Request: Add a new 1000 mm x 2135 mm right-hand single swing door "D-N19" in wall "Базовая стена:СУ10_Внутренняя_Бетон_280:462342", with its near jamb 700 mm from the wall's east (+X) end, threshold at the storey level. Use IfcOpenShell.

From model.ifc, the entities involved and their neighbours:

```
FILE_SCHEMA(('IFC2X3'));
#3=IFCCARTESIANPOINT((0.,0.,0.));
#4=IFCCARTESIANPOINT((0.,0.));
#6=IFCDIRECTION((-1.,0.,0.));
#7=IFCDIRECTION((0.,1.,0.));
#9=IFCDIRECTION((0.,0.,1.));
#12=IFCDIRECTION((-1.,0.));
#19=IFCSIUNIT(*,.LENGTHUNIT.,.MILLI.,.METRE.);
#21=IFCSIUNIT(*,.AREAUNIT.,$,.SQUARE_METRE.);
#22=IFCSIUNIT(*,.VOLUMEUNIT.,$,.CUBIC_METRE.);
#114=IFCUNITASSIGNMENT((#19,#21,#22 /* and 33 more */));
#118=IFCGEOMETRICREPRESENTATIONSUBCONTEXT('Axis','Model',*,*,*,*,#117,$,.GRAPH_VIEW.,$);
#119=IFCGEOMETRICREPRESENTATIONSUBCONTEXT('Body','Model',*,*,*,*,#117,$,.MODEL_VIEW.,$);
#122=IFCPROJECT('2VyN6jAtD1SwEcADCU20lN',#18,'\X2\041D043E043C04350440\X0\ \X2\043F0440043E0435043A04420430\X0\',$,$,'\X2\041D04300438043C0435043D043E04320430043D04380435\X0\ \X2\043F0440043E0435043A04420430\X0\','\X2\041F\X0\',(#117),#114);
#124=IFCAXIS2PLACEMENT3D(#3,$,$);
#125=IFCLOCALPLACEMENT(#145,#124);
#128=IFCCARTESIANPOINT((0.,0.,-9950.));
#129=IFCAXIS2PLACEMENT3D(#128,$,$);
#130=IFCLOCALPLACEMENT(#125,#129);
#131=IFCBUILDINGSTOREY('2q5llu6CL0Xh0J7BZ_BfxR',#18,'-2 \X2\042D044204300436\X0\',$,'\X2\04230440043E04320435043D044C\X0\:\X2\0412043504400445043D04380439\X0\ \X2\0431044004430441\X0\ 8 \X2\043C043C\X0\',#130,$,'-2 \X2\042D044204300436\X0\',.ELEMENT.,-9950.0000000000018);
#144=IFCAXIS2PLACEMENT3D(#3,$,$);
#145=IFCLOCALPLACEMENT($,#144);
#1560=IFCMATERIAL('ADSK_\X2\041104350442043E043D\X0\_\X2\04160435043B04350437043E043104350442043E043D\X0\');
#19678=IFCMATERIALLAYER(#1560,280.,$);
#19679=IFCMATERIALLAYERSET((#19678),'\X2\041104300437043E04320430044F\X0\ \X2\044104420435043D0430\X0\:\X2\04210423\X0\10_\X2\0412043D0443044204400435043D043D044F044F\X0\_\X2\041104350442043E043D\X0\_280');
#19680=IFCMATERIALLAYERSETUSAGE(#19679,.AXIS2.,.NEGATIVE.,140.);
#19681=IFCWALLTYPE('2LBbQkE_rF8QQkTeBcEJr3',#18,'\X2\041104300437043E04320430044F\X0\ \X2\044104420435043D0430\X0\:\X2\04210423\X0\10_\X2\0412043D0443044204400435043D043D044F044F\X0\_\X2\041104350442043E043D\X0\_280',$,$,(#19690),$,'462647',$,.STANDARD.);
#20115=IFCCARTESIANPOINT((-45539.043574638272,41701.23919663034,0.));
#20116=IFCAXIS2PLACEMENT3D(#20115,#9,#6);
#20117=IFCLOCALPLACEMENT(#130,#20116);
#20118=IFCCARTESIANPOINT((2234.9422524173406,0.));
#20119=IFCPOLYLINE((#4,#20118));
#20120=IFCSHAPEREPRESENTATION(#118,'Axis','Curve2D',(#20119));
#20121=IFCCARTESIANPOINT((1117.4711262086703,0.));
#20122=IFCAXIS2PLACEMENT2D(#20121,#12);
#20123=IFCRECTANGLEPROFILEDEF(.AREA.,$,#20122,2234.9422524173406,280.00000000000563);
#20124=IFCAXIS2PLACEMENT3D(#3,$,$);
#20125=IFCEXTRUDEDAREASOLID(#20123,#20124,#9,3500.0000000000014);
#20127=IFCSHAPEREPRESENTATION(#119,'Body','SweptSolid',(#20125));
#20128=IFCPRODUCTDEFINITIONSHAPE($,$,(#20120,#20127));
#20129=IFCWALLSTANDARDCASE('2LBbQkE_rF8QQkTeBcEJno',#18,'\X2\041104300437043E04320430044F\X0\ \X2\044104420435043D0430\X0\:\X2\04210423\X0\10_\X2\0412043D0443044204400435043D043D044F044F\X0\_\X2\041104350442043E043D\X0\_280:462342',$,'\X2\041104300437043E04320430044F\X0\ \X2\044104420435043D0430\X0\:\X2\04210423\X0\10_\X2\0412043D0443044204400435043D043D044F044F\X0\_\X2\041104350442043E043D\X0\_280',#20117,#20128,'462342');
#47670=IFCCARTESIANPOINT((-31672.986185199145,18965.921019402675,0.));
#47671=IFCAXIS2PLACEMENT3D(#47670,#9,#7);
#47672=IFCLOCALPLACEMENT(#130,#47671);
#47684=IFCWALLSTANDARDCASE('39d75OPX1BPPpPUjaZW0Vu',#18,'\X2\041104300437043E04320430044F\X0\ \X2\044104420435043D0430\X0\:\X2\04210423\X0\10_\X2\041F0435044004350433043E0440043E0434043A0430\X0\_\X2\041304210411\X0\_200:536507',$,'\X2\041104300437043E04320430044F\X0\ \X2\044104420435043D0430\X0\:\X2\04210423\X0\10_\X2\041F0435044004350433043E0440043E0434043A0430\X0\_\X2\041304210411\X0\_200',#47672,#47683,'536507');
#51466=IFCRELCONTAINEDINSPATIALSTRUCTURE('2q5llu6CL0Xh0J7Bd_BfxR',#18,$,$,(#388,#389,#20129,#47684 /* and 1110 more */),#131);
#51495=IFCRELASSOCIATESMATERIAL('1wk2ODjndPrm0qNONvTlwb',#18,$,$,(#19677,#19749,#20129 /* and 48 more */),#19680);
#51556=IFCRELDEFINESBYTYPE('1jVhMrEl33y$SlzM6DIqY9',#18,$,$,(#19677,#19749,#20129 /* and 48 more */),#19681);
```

```python
import numpy as np
import ifcopenshell
import ifcopenshell.api.feature
import ifcopenshell.api.geometry
import ifcopenshell.api.root
import ifcopenshell.api.spatial
import ifcopenshell.api.type
import ifcopenshell.geom
import ifcopenshell.util.element
import ifcopenshell.util.placement
import ifcopenshell.util.representation
import ifcopenshell.util.shape
import ifcopenshell.util.unit

model = ifcopenshell.open("model.ifc")
unit_scale = ifcopenshell.util.unit.calculate_unit_scale(model)
settings = ifcopenshell.geom.settings()


def volume(element):
    """Net volume in cubic metres, openings subtracted."""
    shape = ifcopenshell.geom.create_shape(settings, element)
    return ifcopenshell.util.shape.get_volume(shape.geometry)


wall = model.by_guid("2LBbQkE_rF8QQkTeBcEJno")
storey = ifcopenshell.util.element.get_container(wall, ifc_class="IfcBuildingStorey")
context = ifcopenshell.util.representation.get_context(model, "Model", "Body", "MODEL_VIEW")
before = volume(wall)

width, height, from_end, sill = 1, 2.135, 0.7, 0.0  # metres

# The wall runs along its own X axis, and the end named is its -X end.
wall_shape = ifcopenshell.geom.create_shape(settings, wall)
x, y, z = ifcopenshell.util.shape.get_vertices(wall_shape.geometry).T
start = x.min() + from_end
face, thickness = float(y.min()), float(y.max() - y.min())
wall_matrix = ifcopenshell.util.placement.get_local_placement(wall.ObjectPlacement)
level = ifcopenshell.util.placement.get_local_placement(storey.ObjectPlacement)[2, 3]


def in_wall(x, y):
    """Placement at x, y metres in the wall's axes, at sill height."""
    matrix = wall_matrix.copy()
    matrix[:, 3] = wall_matrix @ np.array([x / unit_scale, y / unit_scale, 0.0, 1.0])
    matrix[2, 3] = level + sill / unit_scale
    return matrix


# Opening: a box that overshoots both wall faces by 50 mm.
opening = ifcopenshell.api.root.create_entity(model, ifc_class="IfcOpeningElement")
box = ifcopenshell.api.geometry.add_wall_representation(
    model, context=context, length=width, height=height, thickness=thickness + 0.1
)
ifcopenshell.api.geometry.assign_representation(model, product=opening, representation=box)
ifcopenshell.api.geometry.edit_object_placement(model, product=opening, matrix=in_wall(start, face - 0.05), is_si=False)
ifcopenshell.api.feature.add_feature(model, feature=opening, element=wall)

door = ifcopenshell.api.root.create_entity(model, ifc_class="IfcDoor", name="D-N19")
door.OverallWidth, door.OverallHeight = width / unit_scale, height / unit_scale
body = ifcopenshell.api.geometry.add_door_representation(
    model,
    context=context,
    overall_width=door.OverallWidth,
    overall_height=door.OverallHeight,
    operation_type="SINGLE_SWING_RIGHT",
    lining_properties={"LiningDepth": thickness / unit_scale, "ThresholdDepth": thickness / unit_scale},
)
ifcopenshell.api.geometry.assign_representation(model, product=door, representation=body)
ifcopenshell.api.spatial.assign_container(model, products=[door], relating_structure=storey)
fills = ifcopenshell.api.feature.add_filling(model, opening=opening, element=door)
fills.OwnerHistory = door.OwnerHistory  # required in IFC2X3

# IFC2X3 keeps the operation on the door style.
style = ifcopenshell.api.root.create_entity(model, ifc_class="IfcDoorStyle", name="D-N19")
style.OperationType, style.ConstructionType = "SINGLE_SWING_RIGHT", "NOTDEFINED"
style.ParameterTakesPrecedence = style.Sizeable = False
ifcopenshell.api.type.assign_type(model, related_objects=[door], relating_type=style)

# The lining spans the wall, so the door starts at the wall face.
ifcopenshell.api.geometry.edit_object_placement(model, product=door, matrix=in_wall(start, face), is_si=False)

after = volume(wall)

print(f"wall volume {before:.3f} -> {after:.3f} m3")

model.write("model-out.ifc")
```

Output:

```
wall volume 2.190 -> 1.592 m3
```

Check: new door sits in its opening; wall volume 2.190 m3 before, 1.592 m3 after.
